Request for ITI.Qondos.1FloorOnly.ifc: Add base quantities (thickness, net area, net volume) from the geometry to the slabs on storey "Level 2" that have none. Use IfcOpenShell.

First a look at what the model holds.

```python
import ifcopenshell
import ifcopenshell.util.element
import ifcopenshell.util.unit

model = ifcopenshell.open("ITI.Qondos.1FloorOnly.ifc")
print(model.schema)
for unit_type in ("LENGTHUNIT", "AREAUNIT", "VOLUMEUNIT"):
    print(unit_type, ifcopenshell.util.unit.calculate_unit_scale(model, unit_type))
storey = next(s for s in model.by_type("IfcBuildingStorey") if s.Name == "Level 2")
slabs = [e for e in ifcopenshell.util.element.get_decomposition(storey) if e.is_a("IfcSlab")]
for e in sorted(slabs, key=lambda e: e.id()):
    print(e.id(), e.is_a(), e.Name, list(ifcopenshell.util.element.get_psets(e, qtos_only=True)), sep=" | ")
```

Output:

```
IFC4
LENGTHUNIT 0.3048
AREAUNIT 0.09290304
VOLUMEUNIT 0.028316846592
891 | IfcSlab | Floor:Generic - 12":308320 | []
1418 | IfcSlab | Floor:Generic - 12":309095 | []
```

```python
import ifcopenshell
import ifcopenshell.api.pset
import ifcopenshell.geom
import ifcopenshell.util.element
import ifcopenshell.util.shape
import ifcopenshell.util.unit

model = ifcopenshell.open("ITI.Qondos.1FloorOnly.ifc")
unit_scale = ifcopenshell.util.unit.calculate_unit_scale(model)
area_scale = ifcopenshell.util.unit.calculate_unit_scale(model, "AREAUNIT")
volume_scale = ifcopenshell.util.unit.calculate_unit_scale(model, "VOLUMEUNIT")
settings = ifcopenshell.geom.settings()

storey = next(s for s in model.by_type("IfcBuildingStorey") if s.Name == "Level 2")
slabs = [e for e in ifcopenshell.util.element.get_decomposition(storey) if e.is_a("IfcSlab")]

for e in sorted(slabs, key=lambda e: e.id()):
    if ifcopenshell.util.element.get_psets(e, qtos_only=True, should_inherit=False):
        continue
    # Geometry comes back in metres, in the element's own axes.
    shape = ifcopenshell.geom.create_shape(settings, e)
    values = {
        "Width": ifcopenshell.util.shape.get_z(shape.geometry) / unit_scale,
        "NetArea": ifcopenshell.util.shape.get_footprint_area(shape.geometry) / area_scale,
        "NetVolume": ifcopenshell.util.shape.get_volume(shape.geometry) / volume_scale,
    }
    qto = ifcopenshell.api.pset.add_qto(model, product=e, name="Qto_SlabBaseQuantities")
    ifcopenshell.api.pset.edit_qto(model, qto=qto, properties=values)
    print(e.id(), {k: round(v, 3) for k, v in values.items()})

model.write("ITI.Qondos.1FloorOnly-out.ifc")
```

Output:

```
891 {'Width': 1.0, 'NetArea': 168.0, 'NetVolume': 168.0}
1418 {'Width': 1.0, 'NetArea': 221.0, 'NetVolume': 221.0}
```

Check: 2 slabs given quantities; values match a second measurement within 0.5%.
